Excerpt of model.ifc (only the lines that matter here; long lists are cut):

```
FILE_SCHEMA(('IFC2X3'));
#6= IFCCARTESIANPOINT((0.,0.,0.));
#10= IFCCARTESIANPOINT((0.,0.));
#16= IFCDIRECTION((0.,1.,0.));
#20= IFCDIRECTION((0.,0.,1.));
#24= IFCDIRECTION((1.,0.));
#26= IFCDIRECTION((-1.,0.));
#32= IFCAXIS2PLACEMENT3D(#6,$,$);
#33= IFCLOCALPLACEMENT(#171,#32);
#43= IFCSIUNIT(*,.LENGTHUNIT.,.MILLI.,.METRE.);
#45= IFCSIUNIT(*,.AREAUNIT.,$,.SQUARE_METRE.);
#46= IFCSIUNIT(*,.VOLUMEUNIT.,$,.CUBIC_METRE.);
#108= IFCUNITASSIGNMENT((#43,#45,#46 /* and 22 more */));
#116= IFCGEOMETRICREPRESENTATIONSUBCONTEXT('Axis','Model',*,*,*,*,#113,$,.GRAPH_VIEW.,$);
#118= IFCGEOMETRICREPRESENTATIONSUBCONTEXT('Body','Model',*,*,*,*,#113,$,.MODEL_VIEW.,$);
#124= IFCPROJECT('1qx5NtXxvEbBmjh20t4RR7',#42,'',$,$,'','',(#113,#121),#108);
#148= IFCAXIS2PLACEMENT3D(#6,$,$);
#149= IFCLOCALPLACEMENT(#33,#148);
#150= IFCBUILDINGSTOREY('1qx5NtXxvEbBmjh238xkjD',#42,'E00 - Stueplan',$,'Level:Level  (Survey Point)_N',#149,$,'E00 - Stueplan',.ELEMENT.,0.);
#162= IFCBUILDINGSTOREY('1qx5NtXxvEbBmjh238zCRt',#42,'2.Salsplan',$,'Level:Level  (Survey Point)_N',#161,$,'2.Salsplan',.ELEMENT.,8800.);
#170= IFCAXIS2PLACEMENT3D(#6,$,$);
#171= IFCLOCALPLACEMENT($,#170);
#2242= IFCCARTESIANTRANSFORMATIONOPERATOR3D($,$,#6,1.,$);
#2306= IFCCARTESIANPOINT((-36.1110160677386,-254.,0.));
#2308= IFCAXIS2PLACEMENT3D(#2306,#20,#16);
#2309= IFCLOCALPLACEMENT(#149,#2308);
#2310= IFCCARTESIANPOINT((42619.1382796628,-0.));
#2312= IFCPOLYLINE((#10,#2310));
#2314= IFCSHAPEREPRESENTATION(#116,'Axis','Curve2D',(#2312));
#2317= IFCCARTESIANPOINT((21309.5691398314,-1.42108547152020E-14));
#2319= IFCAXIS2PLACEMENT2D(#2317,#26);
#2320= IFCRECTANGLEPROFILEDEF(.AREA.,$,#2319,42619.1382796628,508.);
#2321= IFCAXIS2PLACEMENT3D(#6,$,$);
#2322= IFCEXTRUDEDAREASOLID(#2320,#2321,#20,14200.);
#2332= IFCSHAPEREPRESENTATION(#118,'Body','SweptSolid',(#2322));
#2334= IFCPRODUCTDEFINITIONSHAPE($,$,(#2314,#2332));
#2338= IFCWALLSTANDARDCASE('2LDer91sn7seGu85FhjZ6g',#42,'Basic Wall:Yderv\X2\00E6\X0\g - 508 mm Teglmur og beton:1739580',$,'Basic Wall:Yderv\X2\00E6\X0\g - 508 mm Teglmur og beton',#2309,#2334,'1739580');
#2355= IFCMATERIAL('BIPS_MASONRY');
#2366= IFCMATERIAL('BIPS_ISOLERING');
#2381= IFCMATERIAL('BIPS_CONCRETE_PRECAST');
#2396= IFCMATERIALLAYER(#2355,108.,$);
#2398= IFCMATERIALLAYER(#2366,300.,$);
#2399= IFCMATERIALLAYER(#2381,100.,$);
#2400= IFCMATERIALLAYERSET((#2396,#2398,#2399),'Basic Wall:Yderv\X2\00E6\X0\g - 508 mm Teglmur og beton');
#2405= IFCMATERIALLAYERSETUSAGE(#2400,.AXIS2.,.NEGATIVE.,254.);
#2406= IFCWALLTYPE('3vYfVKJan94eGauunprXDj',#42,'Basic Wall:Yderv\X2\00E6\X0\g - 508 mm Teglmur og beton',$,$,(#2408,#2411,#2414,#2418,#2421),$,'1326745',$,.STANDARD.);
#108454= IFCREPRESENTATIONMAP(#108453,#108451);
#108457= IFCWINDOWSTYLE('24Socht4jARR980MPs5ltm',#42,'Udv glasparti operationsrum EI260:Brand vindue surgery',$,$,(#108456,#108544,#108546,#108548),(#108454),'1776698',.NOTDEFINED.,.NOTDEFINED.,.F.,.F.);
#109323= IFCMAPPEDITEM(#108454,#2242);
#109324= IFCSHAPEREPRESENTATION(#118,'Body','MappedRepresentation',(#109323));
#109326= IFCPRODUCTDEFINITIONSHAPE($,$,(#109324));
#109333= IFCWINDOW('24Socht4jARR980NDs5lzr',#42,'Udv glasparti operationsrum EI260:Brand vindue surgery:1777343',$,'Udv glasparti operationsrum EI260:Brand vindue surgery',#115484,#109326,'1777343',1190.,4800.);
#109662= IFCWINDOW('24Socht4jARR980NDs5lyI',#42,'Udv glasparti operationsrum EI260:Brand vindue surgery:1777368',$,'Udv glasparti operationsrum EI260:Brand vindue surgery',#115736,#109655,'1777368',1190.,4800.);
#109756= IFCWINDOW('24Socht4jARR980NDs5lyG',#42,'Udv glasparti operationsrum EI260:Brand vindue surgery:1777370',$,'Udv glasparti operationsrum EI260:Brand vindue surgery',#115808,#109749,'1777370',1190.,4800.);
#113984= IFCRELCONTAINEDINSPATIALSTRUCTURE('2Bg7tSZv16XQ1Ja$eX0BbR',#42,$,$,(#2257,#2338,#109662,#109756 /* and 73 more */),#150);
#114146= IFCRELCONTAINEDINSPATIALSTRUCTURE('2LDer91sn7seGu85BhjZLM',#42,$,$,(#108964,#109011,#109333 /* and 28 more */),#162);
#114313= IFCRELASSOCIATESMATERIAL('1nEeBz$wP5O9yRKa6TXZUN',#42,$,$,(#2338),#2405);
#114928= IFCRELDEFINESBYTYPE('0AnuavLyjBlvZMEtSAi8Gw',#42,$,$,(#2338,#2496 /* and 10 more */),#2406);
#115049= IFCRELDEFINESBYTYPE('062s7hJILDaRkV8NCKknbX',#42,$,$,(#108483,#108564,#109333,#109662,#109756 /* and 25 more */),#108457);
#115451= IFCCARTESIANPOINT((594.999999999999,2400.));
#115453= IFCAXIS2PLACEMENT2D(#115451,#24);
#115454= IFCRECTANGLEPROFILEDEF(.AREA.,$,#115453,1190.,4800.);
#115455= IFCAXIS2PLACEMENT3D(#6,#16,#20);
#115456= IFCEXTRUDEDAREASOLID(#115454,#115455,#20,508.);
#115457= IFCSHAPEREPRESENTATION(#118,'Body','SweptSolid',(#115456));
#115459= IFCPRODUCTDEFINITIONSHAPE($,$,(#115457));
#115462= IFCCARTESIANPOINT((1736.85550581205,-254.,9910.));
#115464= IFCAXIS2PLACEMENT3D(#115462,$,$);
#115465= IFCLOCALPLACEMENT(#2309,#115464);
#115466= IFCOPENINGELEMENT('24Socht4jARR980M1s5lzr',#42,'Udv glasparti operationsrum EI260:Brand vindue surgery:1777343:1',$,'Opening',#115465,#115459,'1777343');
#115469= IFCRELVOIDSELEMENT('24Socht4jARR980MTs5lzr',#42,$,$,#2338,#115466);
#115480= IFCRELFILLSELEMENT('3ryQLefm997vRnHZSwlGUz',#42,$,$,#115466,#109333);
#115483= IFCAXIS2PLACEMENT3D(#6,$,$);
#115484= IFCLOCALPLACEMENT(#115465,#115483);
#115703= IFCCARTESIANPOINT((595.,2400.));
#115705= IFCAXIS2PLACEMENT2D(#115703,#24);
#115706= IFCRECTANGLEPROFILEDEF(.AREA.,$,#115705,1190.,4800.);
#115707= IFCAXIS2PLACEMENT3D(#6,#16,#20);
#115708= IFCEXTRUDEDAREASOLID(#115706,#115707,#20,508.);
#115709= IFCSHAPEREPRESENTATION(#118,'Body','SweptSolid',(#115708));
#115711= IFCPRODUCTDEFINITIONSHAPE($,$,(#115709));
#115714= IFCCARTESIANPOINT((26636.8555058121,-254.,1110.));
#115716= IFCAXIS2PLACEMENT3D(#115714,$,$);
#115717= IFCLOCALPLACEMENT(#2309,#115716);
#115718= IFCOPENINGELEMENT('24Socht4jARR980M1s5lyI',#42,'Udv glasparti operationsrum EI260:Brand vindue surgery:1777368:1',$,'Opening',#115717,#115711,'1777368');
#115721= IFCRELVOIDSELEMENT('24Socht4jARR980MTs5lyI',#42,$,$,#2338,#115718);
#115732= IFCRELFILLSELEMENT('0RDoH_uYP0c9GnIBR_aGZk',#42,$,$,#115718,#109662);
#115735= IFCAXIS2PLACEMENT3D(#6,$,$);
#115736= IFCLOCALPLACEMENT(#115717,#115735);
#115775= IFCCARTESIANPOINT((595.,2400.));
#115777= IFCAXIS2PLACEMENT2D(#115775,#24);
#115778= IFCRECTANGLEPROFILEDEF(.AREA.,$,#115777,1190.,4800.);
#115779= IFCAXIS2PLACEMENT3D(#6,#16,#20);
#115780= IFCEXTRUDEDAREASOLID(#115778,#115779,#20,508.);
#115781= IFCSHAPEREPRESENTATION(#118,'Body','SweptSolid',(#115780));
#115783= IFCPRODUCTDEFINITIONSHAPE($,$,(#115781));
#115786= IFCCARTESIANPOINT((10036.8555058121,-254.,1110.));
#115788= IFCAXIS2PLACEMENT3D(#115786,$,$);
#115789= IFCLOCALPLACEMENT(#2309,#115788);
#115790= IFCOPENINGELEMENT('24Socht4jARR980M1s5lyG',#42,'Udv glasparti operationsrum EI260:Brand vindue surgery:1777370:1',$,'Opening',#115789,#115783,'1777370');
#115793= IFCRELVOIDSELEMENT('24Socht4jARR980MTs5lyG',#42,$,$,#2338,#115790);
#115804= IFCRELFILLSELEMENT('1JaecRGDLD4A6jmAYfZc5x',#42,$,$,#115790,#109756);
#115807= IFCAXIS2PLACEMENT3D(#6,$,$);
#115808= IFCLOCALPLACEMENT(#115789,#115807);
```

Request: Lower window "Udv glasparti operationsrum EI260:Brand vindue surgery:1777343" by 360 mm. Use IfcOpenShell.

```python
import numpy as np
import ifcopenshell
import ifcopenshell.api.geometry
import ifcopenshell.util.placement
import ifcopenshell.util.unit

model = ifcopenshell.open("model.ifc")
unit_scale = ifcopenshell.util.unit.calculate_unit_scale(model)

window = model.by_id(109333)
opening = window.FillsVoids[0].RelatingOpeningElement
dz = -0.36 / unit_scale

shift = np.array([0.0, 0.0, dz])
# The window is placed relative to its opening, so it follows when the opening moves.
matrix = ifcopenshell.util.placement.get_local_placement(opening.ObjectPlacement)
matrix[:3, 3] += shift
ifcopenshell.api.geometry.edit_object_placement(
    model, product=opening, matrix=matrix, is_si=False, should_transform_children=True
)

print(f"moved by {dz * unit_scale:+.3f} m")

model.write("model_v2.ifc")
```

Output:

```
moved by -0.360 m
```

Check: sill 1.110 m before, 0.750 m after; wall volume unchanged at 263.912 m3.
